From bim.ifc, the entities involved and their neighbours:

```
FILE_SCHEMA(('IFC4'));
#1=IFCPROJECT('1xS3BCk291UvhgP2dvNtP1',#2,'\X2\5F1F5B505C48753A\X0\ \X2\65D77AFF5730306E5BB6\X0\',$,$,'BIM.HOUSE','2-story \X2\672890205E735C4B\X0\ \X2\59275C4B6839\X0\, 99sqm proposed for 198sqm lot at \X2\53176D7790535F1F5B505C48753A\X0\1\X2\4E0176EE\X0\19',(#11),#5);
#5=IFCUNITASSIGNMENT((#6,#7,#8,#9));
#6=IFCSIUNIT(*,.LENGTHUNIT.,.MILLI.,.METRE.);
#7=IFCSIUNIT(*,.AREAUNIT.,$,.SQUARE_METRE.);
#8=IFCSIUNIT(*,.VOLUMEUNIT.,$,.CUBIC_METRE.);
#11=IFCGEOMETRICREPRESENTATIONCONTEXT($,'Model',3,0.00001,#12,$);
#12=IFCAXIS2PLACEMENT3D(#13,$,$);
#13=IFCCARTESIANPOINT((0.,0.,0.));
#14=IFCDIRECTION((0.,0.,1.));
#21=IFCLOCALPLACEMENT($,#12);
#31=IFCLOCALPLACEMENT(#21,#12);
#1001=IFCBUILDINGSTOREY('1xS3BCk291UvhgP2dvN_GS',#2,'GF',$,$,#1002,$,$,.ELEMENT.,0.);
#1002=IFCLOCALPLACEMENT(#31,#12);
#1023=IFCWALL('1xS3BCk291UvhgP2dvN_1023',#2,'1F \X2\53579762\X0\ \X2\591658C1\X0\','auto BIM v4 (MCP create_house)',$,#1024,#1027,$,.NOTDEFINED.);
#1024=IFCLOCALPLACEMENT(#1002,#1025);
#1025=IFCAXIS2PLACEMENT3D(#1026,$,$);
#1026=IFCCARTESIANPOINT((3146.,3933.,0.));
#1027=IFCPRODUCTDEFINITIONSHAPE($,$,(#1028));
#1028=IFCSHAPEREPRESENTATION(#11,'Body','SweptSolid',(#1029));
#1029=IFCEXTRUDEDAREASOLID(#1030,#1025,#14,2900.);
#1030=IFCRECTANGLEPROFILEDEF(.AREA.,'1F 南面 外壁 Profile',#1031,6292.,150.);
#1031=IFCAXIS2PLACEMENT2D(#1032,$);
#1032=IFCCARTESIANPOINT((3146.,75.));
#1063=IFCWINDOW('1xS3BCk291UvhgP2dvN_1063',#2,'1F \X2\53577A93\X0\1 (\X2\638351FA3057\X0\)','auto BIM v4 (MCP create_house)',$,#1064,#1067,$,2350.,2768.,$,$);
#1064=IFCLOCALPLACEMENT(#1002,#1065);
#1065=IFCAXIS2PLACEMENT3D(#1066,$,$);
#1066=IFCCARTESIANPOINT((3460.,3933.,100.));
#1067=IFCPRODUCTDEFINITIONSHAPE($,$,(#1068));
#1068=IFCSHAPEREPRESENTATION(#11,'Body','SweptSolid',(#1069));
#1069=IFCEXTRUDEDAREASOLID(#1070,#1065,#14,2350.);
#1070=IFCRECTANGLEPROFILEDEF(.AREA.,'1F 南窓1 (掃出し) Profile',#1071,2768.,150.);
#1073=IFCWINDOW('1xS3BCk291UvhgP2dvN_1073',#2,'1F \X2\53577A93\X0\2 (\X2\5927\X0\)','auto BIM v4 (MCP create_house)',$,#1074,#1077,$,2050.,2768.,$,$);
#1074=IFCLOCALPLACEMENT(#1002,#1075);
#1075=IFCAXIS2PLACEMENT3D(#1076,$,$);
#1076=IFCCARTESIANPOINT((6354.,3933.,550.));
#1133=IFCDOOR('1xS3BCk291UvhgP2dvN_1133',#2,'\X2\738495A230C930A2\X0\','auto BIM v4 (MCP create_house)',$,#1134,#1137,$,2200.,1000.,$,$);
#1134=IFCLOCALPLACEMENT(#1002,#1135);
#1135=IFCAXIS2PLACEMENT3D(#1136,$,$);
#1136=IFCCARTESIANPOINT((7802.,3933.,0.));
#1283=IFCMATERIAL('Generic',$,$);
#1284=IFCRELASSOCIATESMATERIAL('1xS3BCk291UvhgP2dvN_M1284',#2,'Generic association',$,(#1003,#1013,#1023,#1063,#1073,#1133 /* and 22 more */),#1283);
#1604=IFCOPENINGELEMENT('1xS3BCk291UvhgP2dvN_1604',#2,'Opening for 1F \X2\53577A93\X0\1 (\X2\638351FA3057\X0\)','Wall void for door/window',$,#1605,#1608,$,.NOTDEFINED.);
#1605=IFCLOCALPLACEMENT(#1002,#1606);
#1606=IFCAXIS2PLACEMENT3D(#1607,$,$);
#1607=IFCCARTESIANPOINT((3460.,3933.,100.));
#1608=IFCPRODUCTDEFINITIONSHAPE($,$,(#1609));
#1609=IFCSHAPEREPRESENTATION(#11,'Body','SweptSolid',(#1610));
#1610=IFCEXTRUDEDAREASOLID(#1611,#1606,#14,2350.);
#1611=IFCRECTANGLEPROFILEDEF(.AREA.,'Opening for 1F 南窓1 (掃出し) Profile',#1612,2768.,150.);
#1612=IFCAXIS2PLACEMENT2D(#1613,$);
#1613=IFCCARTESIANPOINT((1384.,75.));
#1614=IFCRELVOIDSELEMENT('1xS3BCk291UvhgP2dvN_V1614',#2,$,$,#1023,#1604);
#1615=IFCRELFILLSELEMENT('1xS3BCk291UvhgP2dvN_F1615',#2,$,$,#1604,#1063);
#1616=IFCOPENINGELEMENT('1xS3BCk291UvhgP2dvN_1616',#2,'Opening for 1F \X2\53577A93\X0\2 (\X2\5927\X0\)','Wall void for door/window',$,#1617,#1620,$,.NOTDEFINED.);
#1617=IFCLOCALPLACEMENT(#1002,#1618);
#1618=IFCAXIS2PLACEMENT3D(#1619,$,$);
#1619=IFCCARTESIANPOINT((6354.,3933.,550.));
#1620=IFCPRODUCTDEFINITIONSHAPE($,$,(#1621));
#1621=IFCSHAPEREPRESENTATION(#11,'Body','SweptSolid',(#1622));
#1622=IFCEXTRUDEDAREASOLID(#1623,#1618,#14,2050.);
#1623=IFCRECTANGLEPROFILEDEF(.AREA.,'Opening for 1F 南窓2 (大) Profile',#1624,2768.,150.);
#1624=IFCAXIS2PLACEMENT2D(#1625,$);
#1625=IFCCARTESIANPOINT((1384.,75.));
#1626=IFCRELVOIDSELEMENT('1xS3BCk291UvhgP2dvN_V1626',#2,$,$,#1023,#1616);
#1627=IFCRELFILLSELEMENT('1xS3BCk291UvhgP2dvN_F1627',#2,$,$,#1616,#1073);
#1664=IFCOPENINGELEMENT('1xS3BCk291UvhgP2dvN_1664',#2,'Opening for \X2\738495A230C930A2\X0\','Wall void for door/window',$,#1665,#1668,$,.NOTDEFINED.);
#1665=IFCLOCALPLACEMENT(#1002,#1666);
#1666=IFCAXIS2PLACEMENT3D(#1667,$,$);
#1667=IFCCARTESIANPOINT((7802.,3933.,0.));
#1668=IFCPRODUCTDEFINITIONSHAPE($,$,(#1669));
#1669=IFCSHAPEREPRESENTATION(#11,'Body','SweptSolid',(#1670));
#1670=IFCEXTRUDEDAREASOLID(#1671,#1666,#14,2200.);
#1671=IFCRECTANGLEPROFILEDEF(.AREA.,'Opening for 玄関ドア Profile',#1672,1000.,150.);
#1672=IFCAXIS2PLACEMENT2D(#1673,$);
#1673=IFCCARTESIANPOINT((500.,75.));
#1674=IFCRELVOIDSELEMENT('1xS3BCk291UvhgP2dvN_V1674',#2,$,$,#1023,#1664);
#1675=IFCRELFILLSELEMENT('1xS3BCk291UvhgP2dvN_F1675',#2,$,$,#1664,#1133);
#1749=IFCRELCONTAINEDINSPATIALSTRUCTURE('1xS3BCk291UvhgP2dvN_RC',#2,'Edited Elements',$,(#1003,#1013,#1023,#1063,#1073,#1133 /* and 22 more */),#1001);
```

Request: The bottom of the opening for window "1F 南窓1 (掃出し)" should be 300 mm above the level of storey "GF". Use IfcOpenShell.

```python
import numpy as np
import ifcopenshell
import ifcopenshell.api.geometry
import ifcopenshell.geom
import ifcopenshell.util.element
import ifcopenshell.util.placement
import ifcopenshell.util.shape
import ifcopenshell.util.unit

model = ifcopenshell.open("bim.ifc")
unit_scale = ifcopenshell.util.unit.calculate_unit_scale(model)

window = model.by_guid("1xS3BCk291UvhgP2dvN_1063")
opening = window.FillsVoids[0].RelatingOpeningElement
storey = ifcopenshell.util.element.get_container(window, ifc_class="IfcBuildingStorey")
level = ifcopenshell.util.placement.get_local_placement(storey.ObjectPlacement)[2, 3]

# The opening's origin need not be at the sill, so measure its lowest point.
shape = ifcopenshell.geom.create_shape(ifcopenshell.geom.settings(), opening)
bottom = ifcopenshell.util.shape.get_shape_bottom_elevation(shape, shape.geometry) / unit_scale
dz = level + 300.0 - bottom

shift = np.array([0.0, 0.0, dz])
# The window is not placed relative to its opening, so move both.
for product in (opening, window):
    matrix = ifcopenshell.util.placement.get_local_placement(product.ObjectPlacement)
    matrix[:3, 3] += shift
    ifcopenshell.api.geometry.edit_object_placement(model, product=product, matrix=matrix, is_si=False)

print(f"moved by {dz * unit_scale:+.3f} m")

model.write("bim-out.ifc")
```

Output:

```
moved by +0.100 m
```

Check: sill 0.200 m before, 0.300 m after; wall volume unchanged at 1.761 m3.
